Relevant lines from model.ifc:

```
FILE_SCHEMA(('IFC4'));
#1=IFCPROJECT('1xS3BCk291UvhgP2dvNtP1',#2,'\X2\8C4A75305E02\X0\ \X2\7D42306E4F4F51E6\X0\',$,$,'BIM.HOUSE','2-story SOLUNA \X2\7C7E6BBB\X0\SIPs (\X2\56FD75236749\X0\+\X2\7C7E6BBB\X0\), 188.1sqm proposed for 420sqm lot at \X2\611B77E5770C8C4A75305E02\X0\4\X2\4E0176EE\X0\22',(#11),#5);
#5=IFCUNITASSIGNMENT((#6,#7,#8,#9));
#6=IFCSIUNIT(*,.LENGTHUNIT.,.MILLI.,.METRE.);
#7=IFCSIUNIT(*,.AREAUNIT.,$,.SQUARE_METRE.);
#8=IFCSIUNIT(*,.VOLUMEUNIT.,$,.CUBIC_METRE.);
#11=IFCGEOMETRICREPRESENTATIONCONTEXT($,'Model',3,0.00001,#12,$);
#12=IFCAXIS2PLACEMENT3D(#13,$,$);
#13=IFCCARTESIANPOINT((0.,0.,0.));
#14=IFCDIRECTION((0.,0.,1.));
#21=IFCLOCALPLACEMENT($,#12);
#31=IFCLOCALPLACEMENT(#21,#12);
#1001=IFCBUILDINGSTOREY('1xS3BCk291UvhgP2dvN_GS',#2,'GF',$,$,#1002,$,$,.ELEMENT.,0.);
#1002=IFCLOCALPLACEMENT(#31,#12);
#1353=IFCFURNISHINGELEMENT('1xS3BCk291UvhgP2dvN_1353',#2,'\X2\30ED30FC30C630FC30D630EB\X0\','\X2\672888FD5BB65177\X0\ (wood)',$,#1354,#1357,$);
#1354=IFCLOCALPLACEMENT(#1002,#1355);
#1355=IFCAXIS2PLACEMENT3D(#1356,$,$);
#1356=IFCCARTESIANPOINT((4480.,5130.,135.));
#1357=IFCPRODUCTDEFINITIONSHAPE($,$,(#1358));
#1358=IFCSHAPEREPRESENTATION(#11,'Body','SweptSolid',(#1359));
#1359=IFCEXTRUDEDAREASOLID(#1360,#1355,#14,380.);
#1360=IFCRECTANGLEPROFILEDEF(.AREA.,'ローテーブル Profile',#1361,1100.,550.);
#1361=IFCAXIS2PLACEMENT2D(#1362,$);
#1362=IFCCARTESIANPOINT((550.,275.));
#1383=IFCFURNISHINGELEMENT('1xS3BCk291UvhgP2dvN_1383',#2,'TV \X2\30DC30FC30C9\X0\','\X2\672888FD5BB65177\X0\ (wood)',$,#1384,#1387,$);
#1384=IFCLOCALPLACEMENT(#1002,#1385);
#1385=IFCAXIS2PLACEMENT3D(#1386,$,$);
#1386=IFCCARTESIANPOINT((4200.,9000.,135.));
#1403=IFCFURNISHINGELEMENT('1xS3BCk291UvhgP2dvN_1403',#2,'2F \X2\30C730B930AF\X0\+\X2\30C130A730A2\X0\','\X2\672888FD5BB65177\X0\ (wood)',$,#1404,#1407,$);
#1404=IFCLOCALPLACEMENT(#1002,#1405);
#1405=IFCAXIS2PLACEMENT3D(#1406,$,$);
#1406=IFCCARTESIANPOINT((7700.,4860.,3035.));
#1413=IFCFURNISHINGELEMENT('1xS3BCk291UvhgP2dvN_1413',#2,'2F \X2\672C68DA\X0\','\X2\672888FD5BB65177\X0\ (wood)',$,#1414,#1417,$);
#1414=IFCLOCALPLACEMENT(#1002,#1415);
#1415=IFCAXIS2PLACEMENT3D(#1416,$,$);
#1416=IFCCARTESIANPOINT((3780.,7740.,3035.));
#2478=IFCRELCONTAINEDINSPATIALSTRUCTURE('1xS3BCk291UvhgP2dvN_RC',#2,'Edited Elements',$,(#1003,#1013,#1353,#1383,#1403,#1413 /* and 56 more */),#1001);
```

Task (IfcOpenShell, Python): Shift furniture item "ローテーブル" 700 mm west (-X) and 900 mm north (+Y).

```python
import ifcopenshell
import ifcopenshell.api.geometry
import ifcopenshell.util.placement
import ifcopenshell.util.unit

model = ifcopenshell.open("model.ifc")
unit_scale = ifcopenshell.util.unit.calculate_unit_scale(model)

item = model.by_guid("1xS3BCk291UvhgP2dvN_1353")
matrix = ifcopenshell.util.placement.get_local_placement(item.ObjectPlacement)
matrix[0, 3] -= 0.7 / unit_scale
matrix[1, 3] += 0.9 / unit_scale
ifcopenshell.api.geometry.edit_object_placement(model, product=item, matrix=matrix, is_si=False)

print(ifcopenshell.util.placement.get_local_placement(item.ObjectPlacement).round(3) + 0.0)

model.write("model_rev.ifc")
```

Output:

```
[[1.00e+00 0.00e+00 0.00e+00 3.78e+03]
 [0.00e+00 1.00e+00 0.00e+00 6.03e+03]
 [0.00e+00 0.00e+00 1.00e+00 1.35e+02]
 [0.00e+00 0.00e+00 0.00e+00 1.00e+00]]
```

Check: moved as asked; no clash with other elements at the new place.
